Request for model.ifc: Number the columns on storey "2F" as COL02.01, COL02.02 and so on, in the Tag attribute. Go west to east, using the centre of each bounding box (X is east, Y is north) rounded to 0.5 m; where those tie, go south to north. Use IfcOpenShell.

First a look at what the model holds.

```python
import ifcopenshell
import ifcopenshell.util.element
import ifcopenshell.util.placement

model = ifcopenshell.open("model.ifc")
print(model.schema)
storey = next(s for s in model.by_type("IfcBuildingStorey") if s.Name == "2F")
columns = [e for e in ifcopenshell.util.element.get_decomposition(storey) if e.is_a("IfcColumn")]
for e in sorted(columns, key=lambda e: e.id()):
    origin = ifcopenshell.util.placement.get_local_placement(e.ObjectPlacement)[:3, 3]
    print(e.id(), e.Tag, e.Name, origin.round(2) + 0.0, sep=" | ")
```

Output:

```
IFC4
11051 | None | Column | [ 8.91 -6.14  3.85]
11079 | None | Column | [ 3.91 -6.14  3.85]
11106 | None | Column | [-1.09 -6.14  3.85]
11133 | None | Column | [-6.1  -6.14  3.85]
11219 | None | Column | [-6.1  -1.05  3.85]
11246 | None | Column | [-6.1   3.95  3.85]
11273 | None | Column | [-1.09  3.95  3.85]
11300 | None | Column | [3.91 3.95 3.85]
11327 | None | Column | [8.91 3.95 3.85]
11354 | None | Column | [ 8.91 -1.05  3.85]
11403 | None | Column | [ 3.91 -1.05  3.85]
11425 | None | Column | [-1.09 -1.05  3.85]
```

```python
import ifcopenshell
import ifcopenshell.geom
import ifcopenshell.util.element
import ifcopenshell.util.shape

model = ifcopenshell.open("model.ifc")
settings = ifcopenshell.geom.settings()
settings.set("use-world-coords", True)


def centre(element):
    shape = ifcopenshell.geom.create_shape(settings, element)
    return ifcopenshell.util.shape.get_bbox_centroid(shape.geometry)


storey = next(s for s in model.by_type("IfcBuildingStorey") if s.Name == "2F")
columns = [e for e in ifcopenshell.util.element.get_decomposition(storey) if e.is_a("IfcColumn")]

# Insertion points can sit at a corner or the storey origin, so sort by the geometry (in metres).
centres = {e: centre(e) for e in columns}
columns.sort(key=lambda e: (round(centres[e][0] / 0.5), centres[e][1]))

for i, e in enumerate(columns, start=1):
    number = f"COL02.{i:02d}"
    e.Tag = number
    print(e.id(), number)

model.write("model_edited.ifc")
```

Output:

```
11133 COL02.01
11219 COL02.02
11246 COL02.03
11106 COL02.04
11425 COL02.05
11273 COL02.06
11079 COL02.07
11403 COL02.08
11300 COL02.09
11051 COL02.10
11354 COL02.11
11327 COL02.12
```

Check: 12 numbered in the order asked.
